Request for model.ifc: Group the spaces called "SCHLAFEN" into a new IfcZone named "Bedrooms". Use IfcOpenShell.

First a look at what the model holds.

```python
import ifcopenshell

model = ifcopenshell.open("model.ifc")
print(model.schema)
seen = {}
for space in model.by_type("IfcSpace"):
    seen[space.LongName] = seen.get(space.LongName, 0) + 1
for name, count in sorted(seen.items(), key=str):
    print(count, "x", name)
print("zones:", [z.Name for z in model.by_type("IfcZone")][:20])
```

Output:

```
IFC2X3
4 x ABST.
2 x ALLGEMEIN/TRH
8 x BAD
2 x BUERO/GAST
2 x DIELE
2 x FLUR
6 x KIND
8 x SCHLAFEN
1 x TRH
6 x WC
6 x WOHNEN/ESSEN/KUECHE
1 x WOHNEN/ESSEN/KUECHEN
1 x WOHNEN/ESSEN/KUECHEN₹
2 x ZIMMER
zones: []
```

```python
import ifcopenshell
import ifcopenshell.api.group
import ifcopenshell.api.root

model = ifcopenshell.open("model.ifc")

names = {"SCHLAFEN"}
spaces = [s for s in model.by_type("IfcSpace") if s.LongName in names]

zone = ifcopenshell.api.root.create_entity(model, ifc_class="IfcZone", name="Bedrooms")
ifcopenshell.api.group.assign_group(model, products=spaces, group=zone)
print(len(spaces), "spaces in", zone.Name)

model.write("model_rev.ifc")
```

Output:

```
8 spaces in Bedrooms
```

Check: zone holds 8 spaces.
